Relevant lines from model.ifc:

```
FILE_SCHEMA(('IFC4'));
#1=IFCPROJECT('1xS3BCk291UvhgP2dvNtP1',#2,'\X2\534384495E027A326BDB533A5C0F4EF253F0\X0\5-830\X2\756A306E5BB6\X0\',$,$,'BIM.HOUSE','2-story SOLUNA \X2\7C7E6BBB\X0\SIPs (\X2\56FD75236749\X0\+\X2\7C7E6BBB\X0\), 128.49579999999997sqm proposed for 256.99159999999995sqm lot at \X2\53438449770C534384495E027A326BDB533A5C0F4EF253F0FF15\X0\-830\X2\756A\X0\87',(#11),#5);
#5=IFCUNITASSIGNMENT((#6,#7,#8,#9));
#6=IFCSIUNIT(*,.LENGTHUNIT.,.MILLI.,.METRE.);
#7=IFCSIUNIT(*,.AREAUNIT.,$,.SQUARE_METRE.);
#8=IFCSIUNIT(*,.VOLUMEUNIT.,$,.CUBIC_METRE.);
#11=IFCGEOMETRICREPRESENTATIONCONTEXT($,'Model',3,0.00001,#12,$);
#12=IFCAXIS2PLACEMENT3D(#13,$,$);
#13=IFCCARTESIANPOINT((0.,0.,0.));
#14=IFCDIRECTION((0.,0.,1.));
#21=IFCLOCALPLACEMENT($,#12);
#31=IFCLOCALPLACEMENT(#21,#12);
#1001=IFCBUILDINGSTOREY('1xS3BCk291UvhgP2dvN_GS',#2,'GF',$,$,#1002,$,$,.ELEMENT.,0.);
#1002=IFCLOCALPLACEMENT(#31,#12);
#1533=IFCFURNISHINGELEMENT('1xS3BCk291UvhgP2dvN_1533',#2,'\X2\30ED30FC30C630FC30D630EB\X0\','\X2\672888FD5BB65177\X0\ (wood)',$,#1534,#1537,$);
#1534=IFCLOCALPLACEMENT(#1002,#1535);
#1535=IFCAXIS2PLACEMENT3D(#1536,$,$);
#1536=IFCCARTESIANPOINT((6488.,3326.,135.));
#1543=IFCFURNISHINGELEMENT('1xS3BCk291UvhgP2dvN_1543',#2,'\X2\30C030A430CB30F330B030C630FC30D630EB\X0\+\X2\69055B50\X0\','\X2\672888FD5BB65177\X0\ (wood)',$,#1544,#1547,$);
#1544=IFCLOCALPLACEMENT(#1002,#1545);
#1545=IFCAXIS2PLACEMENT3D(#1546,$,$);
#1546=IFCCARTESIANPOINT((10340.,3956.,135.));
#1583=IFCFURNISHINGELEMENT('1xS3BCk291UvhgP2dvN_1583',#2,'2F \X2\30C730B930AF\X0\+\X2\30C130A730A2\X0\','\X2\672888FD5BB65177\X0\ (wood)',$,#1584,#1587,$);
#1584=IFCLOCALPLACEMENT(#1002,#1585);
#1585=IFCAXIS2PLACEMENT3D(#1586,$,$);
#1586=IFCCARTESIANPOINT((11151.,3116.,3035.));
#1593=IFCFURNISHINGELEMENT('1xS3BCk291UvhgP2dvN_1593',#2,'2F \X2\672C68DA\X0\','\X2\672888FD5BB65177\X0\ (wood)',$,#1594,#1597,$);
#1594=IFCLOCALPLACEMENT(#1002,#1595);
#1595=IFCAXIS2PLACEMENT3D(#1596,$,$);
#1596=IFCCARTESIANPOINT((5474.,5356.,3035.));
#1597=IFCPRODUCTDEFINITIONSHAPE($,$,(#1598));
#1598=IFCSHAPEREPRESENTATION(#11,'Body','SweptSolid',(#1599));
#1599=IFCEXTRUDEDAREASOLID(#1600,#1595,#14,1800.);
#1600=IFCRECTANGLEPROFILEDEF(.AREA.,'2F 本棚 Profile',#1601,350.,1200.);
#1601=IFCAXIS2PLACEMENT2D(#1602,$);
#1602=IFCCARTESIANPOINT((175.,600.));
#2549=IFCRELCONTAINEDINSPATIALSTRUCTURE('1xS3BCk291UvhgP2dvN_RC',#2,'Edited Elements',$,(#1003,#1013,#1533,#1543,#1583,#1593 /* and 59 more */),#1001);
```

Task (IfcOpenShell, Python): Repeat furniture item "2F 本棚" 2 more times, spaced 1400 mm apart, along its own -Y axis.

```python
import ifcopenshell
import ifcopenshell.api.geometry
import ifcopenshell.api.root
import ifcopenshell.util.element
import ifcopenshell.util.placement
import ifcopenshell.util.unit

model = ifcopenshell.open("model.ifc")
unit_scale = ifcopenshell.util.unit.calculate_unit_scale(model)


def reuse_history(source, copy):
    """copy_class also copies each property set's owner history, people and application; keep the originals."""
    for rel in copy.IsDefinedBy:
        if rel.is_a("IfcRelDefinesByProperties") and (history := rel.RelatingPropertyDefinition.OwnerHistory):
            rel.RelatingPropertyDefinition.OwnerHistory = source.OwnerHistory
            ifcopenshell.util.element.remove_deep2(model, history)


source = model.by_guid("1xS3BCk291UvhgP2dvN_1593")
base = ifcopenshell.util.placement.get_local_placement(source.ObjectPlacement)
step = -base[:3, 1] * 1.4 / unit_scale

for i in range(1, 3):
    copy = ifcopenshell.api.root.copy_class(model, product=source)
    copy.Representation = ifcopenshell.util.element.copy_deep(
        model, source.Representation, exclude=["IfcGeometricRepresentationContext", "IfcRepresentationMap"]
    )
    reuse_history(source, copy)
    matrix = base.copy()
    matrix[:3, 3] += i * step
    print("added at", matrix[:3, 3].round(3) + 0.0)
    ifcopenshell.api.geometry.edit_object_placement(model, product=copy, matrix=matrix, is_si=False)

model.write("model_v2.ifc")
```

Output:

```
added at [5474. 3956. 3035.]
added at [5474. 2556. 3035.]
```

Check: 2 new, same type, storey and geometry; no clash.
